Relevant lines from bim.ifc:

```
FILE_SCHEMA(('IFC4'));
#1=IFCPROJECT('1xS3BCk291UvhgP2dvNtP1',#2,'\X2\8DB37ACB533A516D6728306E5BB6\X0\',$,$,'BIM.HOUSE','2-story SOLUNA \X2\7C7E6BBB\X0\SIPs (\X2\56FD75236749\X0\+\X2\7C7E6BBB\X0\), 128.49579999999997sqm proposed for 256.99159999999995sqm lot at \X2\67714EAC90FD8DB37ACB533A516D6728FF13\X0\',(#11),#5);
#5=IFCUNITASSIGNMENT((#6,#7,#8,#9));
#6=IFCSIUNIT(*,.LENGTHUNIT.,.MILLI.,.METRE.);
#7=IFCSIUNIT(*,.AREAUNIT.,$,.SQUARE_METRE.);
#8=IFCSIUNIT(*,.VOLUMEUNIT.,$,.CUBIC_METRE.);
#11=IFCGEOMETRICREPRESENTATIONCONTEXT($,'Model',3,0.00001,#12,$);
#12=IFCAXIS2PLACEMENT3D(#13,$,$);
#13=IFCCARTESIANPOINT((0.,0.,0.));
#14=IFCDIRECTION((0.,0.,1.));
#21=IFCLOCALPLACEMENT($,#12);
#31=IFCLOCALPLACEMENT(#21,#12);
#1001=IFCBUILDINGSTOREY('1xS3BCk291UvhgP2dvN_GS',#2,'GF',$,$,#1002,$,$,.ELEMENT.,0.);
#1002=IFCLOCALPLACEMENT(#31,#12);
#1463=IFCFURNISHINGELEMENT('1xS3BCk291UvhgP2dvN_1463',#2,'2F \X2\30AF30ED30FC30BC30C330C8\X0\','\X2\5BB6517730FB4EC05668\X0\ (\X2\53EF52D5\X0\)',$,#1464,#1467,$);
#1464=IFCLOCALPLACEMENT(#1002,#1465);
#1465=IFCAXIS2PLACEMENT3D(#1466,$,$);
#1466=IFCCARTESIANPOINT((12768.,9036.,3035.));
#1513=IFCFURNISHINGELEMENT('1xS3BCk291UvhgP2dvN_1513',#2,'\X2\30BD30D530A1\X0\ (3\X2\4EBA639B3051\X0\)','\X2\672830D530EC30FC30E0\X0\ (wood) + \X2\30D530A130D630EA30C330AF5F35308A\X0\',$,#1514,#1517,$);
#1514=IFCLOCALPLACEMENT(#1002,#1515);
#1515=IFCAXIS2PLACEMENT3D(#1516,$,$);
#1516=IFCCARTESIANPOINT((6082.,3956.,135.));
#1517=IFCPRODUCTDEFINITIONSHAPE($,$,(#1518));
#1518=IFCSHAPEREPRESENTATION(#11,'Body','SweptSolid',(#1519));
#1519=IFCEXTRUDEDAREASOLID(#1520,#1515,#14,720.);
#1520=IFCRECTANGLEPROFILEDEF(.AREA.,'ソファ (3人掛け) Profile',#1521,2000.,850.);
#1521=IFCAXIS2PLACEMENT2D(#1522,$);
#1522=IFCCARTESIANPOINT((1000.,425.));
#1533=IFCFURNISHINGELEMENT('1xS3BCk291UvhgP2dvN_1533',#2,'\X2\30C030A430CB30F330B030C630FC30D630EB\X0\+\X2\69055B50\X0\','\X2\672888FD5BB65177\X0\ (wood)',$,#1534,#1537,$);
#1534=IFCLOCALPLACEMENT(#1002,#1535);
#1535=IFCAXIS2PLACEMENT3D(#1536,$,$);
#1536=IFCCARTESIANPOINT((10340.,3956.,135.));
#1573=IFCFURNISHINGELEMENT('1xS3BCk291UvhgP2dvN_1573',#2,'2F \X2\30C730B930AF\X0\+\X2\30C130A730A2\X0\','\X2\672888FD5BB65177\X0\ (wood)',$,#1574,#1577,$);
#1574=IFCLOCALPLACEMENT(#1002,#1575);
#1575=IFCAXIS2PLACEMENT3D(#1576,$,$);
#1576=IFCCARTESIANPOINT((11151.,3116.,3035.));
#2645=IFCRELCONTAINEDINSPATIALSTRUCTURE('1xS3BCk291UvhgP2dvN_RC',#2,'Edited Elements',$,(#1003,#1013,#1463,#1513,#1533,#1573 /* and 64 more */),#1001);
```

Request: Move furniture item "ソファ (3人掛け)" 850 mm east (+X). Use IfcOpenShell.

```python
import ifcopenshell
import ifcopenshell.api.geometry
import ifcopenshell.util.placement

model = ifcopenshell.open("bim.ifc")

item = model.by_guid("1xS3BCk291UvhgP2dvN_1513")
matrix = ifcopenshell.util.placement.get_local_placement(item.ObjectPlacement)
matrix[0, 3] += 850.0
ifcopenshell.api.geometry.edit_object_placement(model, product=item, matrix=matrix, is_si=False)

print(ifcopenshell.util.placement.get_local_placement(item.ObjectPlacement).round(3) + 0.0)

model.write("bim-out.ifc")
```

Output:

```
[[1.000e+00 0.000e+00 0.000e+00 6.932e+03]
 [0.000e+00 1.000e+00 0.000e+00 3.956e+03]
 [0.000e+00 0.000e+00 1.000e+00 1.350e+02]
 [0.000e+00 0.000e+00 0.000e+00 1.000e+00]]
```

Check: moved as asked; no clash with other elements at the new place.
